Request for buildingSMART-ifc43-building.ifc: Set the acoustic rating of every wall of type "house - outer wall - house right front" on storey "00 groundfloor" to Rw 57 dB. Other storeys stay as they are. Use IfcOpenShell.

First a look at what the model holds.

```python
import ifcopenshell
import ifcopenshell.util.element

model = ifcopenshell.open("buildingSMART-ifc43-building.ifc")
print(model.schema)
storey = next(s for s in model.by_type("IfcBuildingStorey") if s.Name == "00 groundfloor")
walls = [e for e in ifcopenshell.util.element.get_decomposition(storey) if e.is_a("IfcWall")]
seen = {}
for e in walls:
    element_type = ifcopenshell.util.element.get_type(e)
    key = (element_type.Name if element_type != e and element_type else None, ifcopenshell.util.element.get_pset(e, "Pset_WallCommon", "AcousticRating"))
    seen[key] = seen.get(key, 0) + 1
for (name, value), count in sorted(seen.items(), key=str):
    print(count, "x", name, "|", value)
```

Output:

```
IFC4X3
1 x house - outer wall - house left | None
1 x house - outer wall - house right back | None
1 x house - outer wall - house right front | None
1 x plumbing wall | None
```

```python
import ifcopenshell
import ifcopenshell.api.pset
import ifcopenshell.util.element

model = ifcopenshell.open("buildingSMART-ifc43-building.ifc")

storey = next(s for s in model.by_type("IfcBuildingStorey") if s.Name == "00 groundfloor")
walls = [e for e in ifcopenshell.util.element.get_decomposition(storey) if e.is_a("IfcWall")]

count = 0
for e in walls:
    element_type = ifcopenshell.util.element.get_type(e)
    if element_type in (None, e) or element_type.Name != "house - outer wall - house right front":
        continue
    # add_pset returns the element's existing set when there is one.
    pset = ifcopenshell.api.pset.add_pset(model, product=e, name="Pset_WallCommon")
    ifcopenshell.api.pset.edit_pset(model, pset=pset, properties={"AcousticRating": "Rw 57 dB"})
    count += 1

print(count, "walls updated")

model.write("buildingSMART-ifc43-building_rev.ifc")
```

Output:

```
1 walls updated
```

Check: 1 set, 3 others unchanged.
